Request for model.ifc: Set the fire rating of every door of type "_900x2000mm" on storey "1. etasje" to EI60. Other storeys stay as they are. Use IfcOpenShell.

First a look at what the model holds.

```python
import ifcopenshell
import ifcopenshell.util.element

model = ifcopenshell.open("model.ifc")
print(model.schema)
storey = next(s for s in model.by_type("IfcBuildingStorey") if s.Name == "1. etasje")
doors = [e for e in ifcopenshell.util.element.get_decomposition(storey) if e.is_a("IfcDoor")]
seen = {}
for e in doors:
    element_type = ifcopenshell.util.element.get_type(e)
    key = (element_type.Name if element_type != e and element_type else None, ifcopenshell.util.element.get_pset(e, "Pset_DoorCommon", "FireRating"))
    seen[key] = seen.get(key, 0) + 1
for (name, value), count in sorted(seen.items(), key=str):
    print(count, "x", name, "|", value)
```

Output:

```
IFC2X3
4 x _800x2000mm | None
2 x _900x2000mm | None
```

```python
import ifcopenshell
import ifcopenshell.api.pset
import ifcopenshell.util.element

model = ifcopenshell.open("model.ifc")

storey = next(s for s in model.by_type("IfcBuildingStorey") if s.Name == "1. etasje")
doors = [e for e in ifcopenshell.util.element.get_decomposition(storey) if e.is_a("IfcDoor")]

count = 0
for e in doors:
    element_type = ifcopenshell.util.element.get_type(e)
    if element_type in (None, e) or element_type.Name != "_900x2000mm":
        continue
    # add_pset returns the element's existing set when there is one.
    pset = ifcopenshell.api.pset.add_pset(model, product=e, name="Pset_DoorCommon")
    ifcopenshell.api.pset.edit_pset(model, pset=pset, properties={"FireRating": "EI60"})
    count += 1

print(count, "doors updated")

model.write("model_rev.ifc")
```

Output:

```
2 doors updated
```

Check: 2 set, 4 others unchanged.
